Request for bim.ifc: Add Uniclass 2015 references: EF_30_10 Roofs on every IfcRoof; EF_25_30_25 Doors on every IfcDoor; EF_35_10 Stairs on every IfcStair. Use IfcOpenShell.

First a look at what the model holds.

```python
import ifcopenshell

model = ifcopenshell.open("bim.ifc")
print(model.schema)
print("classifications:", [c.Name for c in model.by_type("IfcClassification")])
for ifc_class in ("IfcDoor", "IfcRoof", "IfcStair", "IfcWall", "IfcWindow"):
    print(ifc_class, len(model.by_type(ifc_class)))
```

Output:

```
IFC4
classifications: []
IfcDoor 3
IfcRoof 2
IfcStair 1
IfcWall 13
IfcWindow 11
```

```python
import ifcopenshell
import ifcopenshell.api.classification

model = ifcopenshell.open("bim.ifc")

system = ifcopenshell.api.classification.add_classification(model, classification="Uniclass 2015")

codes = {
    "IfcRoof": ("EF_30_10", "Roofs"),
    "IfcDoor": ("EF_25_30_25", "Doors"),
    "IfcStair": ("EF_35_10", "Stairs"),
}
for ifc_class, (code, name) in codes.items():
    products = model.by_type(ifc_class)
    ifcopenshell.api.classification.add_reference(
        model, products=products, classification=system, identification=code, name=name
    )
    print(code, len(products))

model.write("bim_edited.ifc")
```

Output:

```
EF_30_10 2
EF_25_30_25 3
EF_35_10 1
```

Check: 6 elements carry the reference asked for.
